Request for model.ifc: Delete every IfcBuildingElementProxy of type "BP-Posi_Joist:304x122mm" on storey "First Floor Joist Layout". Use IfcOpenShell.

First a look at what the model holds.

```python
import ifcopenshell
import ifcopenshell.util.element

model = ifcopenshell.open("model.ifc")
print(model.schema)
storey = next(s for s in model.by_type("IfcBuildingStorey") if s.Name == "First Floor Joist Layout")
proxies = [e for e in ifcopenshell.util.element.get_decomposition(storey) if e.is_a("IfcBuildingElementProxy")]
seen = {}
for e in proxies:
    element_type = ifcopenshell.util.element.get_type(e)
    name = element_type.Name if element_type not in (None, e) else None
    seen[name] = seen.get(name, 0) + 1
for name, count in sorted(seen.items(), key=str):
    print(count, "x", name)
```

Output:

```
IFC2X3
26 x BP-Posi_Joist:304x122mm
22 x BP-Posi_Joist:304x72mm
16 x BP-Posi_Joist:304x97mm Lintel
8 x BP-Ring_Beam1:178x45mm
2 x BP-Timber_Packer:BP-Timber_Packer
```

```python
import ifcopenshell
import ifcopenshell.api.root
import ifcopenshell.util.element

model = ifcopenshell.open("model.ifc")

storey = next(s for s in model.by_type("IfcBuildingStorey") if s.Name == "First Floor Joist Layout")
proxies = [e for e in ifcopenshell.util.element.get_decomposition(storey) if e.is_a("IfcBuildingElementProxy")]
targets = [e for e in proxies if (t := ifcopenshell.util.element.get_type(e)) not in (None, e) and t.Name == "BP-Posi_Joist:304x122mm"]

for e in targets:
    ifcopenshell.api.root.remove_product(model, product=e)
print(len(targets), "removed")

model.write("model_rev.ifc")
```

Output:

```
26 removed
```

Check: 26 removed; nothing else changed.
